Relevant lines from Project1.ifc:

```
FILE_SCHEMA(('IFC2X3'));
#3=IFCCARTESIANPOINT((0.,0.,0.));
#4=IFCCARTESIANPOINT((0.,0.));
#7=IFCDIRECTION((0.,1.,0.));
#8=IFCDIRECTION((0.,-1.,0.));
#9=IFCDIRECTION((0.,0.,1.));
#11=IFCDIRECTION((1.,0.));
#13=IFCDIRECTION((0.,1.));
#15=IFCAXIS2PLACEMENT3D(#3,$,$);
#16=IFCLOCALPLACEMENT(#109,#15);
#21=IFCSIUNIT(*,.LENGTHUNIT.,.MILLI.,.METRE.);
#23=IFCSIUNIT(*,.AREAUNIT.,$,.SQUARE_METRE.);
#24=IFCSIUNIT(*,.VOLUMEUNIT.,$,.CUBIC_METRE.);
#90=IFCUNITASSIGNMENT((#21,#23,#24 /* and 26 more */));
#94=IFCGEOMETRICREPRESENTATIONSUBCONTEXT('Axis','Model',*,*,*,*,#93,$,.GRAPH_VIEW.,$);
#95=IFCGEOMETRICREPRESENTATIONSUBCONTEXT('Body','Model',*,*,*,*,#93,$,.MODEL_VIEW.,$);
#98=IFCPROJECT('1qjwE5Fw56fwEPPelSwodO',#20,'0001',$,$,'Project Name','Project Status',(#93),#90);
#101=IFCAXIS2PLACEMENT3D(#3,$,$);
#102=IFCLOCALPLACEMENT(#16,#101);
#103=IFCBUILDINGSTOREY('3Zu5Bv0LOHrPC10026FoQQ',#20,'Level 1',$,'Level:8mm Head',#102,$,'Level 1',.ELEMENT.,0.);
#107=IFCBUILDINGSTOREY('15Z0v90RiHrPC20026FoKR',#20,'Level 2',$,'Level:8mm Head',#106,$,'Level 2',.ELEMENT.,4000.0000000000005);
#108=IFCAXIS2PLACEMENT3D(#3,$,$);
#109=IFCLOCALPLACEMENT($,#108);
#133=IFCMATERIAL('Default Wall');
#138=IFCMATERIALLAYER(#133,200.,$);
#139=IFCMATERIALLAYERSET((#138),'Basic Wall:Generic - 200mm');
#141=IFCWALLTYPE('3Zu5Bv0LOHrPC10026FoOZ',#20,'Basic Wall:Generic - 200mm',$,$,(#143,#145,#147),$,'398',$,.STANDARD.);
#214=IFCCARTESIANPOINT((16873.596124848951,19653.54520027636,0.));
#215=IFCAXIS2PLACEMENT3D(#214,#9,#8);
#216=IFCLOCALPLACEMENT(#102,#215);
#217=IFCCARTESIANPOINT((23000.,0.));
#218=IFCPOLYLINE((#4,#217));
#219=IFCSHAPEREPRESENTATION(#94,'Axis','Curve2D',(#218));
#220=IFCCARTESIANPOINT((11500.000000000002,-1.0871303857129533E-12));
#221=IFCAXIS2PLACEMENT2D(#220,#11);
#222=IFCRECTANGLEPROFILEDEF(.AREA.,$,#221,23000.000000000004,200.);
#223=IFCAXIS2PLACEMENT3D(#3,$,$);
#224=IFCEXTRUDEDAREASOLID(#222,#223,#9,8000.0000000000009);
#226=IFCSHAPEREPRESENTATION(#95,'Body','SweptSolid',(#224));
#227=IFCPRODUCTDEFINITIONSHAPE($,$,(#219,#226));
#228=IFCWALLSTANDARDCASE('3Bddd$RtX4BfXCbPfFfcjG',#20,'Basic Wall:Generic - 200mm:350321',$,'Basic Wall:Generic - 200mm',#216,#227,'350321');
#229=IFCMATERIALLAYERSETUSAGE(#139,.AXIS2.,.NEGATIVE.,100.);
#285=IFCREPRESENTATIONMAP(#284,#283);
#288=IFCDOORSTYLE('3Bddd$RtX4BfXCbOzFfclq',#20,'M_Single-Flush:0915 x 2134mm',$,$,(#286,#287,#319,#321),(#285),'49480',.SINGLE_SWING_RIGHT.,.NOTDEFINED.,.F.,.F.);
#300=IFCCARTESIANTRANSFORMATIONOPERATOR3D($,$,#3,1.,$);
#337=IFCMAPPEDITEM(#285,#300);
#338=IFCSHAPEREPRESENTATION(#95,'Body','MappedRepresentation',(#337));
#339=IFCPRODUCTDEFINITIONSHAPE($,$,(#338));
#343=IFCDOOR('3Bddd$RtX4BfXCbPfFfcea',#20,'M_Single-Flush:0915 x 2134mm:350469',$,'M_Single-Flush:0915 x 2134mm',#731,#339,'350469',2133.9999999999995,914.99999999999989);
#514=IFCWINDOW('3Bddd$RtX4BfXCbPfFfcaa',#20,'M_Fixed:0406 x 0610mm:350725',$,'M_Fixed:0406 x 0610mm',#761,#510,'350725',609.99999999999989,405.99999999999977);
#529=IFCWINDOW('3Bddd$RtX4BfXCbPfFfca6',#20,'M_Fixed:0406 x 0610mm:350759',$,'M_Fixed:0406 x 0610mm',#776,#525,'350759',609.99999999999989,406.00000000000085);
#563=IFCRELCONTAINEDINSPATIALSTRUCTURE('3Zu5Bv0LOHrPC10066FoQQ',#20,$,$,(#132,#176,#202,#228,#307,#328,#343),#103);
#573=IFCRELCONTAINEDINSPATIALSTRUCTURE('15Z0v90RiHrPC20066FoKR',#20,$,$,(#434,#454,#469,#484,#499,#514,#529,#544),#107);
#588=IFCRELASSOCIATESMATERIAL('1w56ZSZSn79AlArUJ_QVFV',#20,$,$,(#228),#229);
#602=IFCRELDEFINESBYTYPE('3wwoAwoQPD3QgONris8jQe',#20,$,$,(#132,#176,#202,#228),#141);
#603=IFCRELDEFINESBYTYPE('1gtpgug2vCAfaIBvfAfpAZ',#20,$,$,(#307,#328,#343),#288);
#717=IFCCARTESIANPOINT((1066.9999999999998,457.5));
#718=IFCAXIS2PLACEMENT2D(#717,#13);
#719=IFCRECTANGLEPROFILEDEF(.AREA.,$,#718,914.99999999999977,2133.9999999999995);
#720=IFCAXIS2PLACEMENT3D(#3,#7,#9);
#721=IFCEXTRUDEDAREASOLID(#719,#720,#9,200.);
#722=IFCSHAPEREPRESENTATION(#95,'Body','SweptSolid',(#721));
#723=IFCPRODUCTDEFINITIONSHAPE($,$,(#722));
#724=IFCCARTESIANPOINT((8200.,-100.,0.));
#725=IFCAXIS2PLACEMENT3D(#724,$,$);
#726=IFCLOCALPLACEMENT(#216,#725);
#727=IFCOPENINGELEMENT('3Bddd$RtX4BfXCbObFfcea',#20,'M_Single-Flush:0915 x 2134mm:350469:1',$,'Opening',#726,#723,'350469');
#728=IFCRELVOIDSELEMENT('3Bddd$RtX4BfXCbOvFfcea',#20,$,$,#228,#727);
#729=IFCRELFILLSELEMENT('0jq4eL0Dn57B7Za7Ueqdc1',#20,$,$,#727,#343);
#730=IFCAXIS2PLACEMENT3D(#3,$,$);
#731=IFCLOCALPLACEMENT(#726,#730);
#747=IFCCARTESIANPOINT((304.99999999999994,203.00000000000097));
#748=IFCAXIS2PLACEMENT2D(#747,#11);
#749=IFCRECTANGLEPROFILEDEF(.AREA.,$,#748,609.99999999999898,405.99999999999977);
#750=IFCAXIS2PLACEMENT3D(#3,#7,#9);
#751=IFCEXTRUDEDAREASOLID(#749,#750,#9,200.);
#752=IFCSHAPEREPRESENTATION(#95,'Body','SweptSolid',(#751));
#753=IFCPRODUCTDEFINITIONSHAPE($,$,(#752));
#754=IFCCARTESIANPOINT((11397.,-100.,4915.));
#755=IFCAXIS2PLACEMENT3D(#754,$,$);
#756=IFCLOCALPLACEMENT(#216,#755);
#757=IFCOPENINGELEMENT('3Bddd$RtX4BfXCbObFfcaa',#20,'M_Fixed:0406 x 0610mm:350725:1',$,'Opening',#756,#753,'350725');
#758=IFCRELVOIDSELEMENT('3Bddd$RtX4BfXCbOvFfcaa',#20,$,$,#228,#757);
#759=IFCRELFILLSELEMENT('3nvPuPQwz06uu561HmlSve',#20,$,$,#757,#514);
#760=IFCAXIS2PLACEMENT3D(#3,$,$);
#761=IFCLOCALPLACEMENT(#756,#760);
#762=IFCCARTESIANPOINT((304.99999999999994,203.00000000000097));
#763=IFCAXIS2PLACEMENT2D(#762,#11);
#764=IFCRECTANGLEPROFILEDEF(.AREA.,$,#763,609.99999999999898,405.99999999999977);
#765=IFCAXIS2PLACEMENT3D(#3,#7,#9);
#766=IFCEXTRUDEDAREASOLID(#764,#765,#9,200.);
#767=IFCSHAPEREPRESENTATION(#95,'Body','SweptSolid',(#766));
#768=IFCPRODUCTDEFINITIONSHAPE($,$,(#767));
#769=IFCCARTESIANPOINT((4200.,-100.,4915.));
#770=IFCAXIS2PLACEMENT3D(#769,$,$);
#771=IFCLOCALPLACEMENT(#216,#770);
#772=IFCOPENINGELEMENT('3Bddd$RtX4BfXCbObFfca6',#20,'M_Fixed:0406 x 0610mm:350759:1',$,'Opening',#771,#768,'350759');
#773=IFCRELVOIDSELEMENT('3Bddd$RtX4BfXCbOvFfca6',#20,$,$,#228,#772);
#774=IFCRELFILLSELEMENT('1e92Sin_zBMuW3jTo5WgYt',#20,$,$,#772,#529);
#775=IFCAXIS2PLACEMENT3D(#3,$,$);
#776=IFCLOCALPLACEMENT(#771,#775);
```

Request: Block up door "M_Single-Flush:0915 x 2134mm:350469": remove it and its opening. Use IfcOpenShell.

```python
import ifcopenshell
import ifcopenshell.api.feature
import ifcopenshell.api.root
import ifcopenshell.geom
import ifcopenshell.util.shape

model = ifcopenshell.open("Project1.ifc")
settings = ifcopenshell.geom.settings()


def volume(element):
    """Net volume in cubic metres, openings subtracted."""
    shape = ifcopenshell.geom.create_shape(settings, element)
    return ifcopenshell.util.shape.get_volume(shape.geometry)


door = model.by_id(343)
opening = door.FillsVoids[0].RelatingOpeningElement
wall = opening.VoidsElements[0].RelatingBuildingElement
before = volume(wall)

ifcopenshell.api.root.remove_product(model, product=door)
ifcopenshell.api.feature.remove_feature(model, feature=opening)

after = volume(wall)

print(f"wall volume {before:.3f} -> {after:.3f} m3")

model.write("Project1_updated.ifc")
```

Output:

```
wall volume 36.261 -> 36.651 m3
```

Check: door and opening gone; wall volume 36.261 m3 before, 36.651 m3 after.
